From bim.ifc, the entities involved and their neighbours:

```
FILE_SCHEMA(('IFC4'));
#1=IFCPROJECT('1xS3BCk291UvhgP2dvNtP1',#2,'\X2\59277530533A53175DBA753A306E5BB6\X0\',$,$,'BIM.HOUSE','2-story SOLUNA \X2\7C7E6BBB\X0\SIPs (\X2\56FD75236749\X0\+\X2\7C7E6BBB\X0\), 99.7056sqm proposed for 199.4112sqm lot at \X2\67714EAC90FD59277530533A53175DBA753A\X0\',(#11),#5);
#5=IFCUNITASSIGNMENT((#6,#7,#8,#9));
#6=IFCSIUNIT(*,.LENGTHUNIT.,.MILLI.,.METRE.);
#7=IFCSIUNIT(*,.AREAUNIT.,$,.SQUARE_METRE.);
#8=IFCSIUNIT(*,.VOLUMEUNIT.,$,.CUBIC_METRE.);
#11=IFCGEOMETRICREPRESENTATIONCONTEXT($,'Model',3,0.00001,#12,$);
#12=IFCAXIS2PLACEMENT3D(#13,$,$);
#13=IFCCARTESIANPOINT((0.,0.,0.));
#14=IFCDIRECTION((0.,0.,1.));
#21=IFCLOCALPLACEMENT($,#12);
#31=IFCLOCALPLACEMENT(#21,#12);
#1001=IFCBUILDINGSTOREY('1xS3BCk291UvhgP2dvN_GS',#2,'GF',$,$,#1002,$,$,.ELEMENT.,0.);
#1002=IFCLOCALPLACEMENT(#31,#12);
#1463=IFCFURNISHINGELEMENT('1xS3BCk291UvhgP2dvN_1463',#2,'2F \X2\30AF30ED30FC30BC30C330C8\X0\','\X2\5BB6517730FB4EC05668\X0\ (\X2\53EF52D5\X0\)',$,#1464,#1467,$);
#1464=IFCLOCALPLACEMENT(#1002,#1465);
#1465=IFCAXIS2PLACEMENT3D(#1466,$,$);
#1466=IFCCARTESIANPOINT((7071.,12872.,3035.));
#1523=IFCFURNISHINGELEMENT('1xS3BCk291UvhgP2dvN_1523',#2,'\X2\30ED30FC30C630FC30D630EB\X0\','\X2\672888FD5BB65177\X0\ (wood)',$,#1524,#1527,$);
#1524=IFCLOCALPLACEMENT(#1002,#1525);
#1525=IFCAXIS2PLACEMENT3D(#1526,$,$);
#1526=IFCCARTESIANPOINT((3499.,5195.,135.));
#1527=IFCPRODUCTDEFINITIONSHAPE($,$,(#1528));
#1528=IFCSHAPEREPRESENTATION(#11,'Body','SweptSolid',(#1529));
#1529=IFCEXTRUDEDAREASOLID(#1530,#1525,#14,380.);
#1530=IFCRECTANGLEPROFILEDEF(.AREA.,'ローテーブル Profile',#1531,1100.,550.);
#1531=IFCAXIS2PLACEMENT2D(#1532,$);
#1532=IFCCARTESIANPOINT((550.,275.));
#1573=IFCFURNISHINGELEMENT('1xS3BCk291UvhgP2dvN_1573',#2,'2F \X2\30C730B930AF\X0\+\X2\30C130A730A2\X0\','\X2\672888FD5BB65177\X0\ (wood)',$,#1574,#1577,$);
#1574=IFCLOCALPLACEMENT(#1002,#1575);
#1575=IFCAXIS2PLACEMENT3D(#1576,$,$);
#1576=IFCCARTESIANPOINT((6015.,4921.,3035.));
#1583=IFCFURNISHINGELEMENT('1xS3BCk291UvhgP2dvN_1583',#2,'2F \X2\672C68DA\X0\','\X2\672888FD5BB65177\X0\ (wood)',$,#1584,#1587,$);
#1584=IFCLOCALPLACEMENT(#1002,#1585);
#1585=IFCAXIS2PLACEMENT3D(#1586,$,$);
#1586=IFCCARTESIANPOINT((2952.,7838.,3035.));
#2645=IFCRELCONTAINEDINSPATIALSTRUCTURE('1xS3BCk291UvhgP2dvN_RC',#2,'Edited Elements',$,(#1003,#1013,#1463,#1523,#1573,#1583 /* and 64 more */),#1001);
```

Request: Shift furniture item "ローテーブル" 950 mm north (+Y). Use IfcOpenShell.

```python
import ifcopenshell
import ifcopenshell.api.geometry
import ifcopenshell.util.placement

model = ifcopenshell.open("bim.ifc")

item = model.by_guid("1xS3BCk291UvhgP2dvN_1523")
matrix = ifcopenshell.util.placement.get_local_placement(item.ObjectPlacement)
matrix[1, 3] += 950.0
ifcopenshell.api.geometry.edit_object_placement(model, product=item, matrix=matrix, is_si=False)

print(ifcopenshell.util.placement.get_local_placement(item.ObjectPlacement).round(3) + 0.0)

model.write("bim_rev.ifc")
```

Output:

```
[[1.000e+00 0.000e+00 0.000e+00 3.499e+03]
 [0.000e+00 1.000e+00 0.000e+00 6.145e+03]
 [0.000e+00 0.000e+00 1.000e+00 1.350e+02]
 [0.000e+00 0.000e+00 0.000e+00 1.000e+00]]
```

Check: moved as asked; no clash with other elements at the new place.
